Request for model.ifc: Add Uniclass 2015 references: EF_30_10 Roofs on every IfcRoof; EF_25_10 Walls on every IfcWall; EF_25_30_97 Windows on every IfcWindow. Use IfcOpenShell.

First a look at what the model holds.

```python
import ifcopenshell

model = ifcopenshell.open("model.ifc")
print(model.schema)
print("classifications:", [c.Name for c in model.by_type("IfcClassification")])
for ifc_class in ("IfcDoor", "IfcRoof", "IfcStair", "IfcWall", "IfcWindow"):
    print(ifc_class, len(model.by_type(ifc_class)))
```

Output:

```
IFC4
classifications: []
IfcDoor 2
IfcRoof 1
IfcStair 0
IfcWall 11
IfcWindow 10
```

```python
import ifcopenshell
import ifcopenshell.api.classification

model = ifcopenshell.open("model.ifc")

system = ifcopenshell.api.classification.add_classification(model, classification="Uniclass 2015")

codes = {
    "IfcRoof": ("EF_30_10", "Roofs"),
    "IfcWall": ("EF_25_10", "Walls"),
    "IfcWindow": ("EF_25_30_97", "Windows"),
}
for ifc_class, (code, name) in codes.items():
    products = model.by_type(ifc_class)
    ifcopenshell.api.classification.add_reference(
        model, products=products, classification=system, identification=code, name=name
    )
    print(code, len(products))

model.write("model_rev.ifc")
```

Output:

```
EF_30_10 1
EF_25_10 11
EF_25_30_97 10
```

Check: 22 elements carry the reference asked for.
